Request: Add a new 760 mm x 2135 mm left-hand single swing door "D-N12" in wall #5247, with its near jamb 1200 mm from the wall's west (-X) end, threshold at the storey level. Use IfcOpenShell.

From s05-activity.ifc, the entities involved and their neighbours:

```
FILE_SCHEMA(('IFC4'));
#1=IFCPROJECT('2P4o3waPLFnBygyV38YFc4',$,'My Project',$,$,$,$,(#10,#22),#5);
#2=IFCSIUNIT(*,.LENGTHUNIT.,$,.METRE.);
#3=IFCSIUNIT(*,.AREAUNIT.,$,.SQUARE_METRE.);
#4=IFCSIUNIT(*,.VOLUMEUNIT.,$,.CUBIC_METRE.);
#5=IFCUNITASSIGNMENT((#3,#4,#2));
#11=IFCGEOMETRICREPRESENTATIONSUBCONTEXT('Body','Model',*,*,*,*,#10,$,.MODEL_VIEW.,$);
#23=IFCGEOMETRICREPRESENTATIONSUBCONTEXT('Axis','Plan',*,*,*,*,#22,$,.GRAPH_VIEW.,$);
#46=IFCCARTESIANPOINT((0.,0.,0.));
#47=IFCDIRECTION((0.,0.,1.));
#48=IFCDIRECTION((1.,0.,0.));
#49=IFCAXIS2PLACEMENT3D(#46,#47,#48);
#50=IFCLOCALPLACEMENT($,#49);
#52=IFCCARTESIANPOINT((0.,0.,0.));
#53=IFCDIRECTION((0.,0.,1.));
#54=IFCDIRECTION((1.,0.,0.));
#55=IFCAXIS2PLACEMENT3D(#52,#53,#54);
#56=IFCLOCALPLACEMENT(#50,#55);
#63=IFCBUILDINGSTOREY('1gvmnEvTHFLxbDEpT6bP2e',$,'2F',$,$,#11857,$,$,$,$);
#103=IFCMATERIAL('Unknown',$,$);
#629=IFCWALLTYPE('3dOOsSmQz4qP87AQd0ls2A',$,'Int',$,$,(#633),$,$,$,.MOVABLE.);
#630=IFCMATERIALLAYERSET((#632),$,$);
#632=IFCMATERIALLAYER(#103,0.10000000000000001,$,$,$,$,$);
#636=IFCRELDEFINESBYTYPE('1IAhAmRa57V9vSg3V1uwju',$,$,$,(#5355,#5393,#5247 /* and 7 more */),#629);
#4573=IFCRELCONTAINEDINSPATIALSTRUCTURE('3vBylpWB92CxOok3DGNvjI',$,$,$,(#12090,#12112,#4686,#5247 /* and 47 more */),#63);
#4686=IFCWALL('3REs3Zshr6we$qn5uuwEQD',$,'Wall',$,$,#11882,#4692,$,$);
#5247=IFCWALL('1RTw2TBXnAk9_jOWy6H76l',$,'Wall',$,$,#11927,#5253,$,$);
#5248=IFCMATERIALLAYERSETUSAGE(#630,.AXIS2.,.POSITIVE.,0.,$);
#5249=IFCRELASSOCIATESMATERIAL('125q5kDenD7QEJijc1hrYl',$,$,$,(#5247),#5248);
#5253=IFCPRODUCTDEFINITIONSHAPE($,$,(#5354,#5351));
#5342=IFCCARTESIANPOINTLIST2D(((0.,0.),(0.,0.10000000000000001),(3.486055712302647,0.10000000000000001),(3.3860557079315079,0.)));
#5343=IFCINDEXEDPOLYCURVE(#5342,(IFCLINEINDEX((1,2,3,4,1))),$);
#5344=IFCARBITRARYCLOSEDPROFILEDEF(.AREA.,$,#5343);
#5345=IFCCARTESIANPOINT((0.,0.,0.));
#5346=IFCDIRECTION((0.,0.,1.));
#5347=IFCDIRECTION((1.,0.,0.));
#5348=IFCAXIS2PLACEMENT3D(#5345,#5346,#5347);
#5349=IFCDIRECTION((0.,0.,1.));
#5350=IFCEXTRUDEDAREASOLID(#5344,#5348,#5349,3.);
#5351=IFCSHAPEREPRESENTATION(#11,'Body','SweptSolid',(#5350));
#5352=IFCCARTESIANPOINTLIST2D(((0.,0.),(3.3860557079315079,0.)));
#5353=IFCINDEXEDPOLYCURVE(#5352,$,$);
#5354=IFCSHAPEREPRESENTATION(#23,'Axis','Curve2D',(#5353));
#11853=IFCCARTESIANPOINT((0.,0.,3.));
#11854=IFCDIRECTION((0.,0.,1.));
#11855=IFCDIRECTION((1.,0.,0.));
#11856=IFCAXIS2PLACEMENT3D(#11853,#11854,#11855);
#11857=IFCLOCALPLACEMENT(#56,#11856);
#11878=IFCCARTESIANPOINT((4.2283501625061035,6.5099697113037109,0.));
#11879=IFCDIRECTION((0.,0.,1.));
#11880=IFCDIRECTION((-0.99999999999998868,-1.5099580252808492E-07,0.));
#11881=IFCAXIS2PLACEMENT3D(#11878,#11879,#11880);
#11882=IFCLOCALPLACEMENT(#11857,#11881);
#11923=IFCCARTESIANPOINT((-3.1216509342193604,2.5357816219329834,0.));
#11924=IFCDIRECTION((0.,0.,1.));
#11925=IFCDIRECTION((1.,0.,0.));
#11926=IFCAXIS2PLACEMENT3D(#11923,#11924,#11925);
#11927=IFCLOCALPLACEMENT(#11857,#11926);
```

```python
import numpy as np
import ifcopenshell
import ifcopenshell.api.feature
import ifcopenshell.api.geometry
import ifcopenshell.api.root
import ifcopenshell.api.spatial
import ifcopenshell.geom
import ifcopenshell.util.element
import ifcopenshell.util.placement
import ifcopenshell.util.representation
import ifcopenshell.util.shape
import ifcopenshell.util.unit

model = ifcopenshell.open("s05-activity.ifc")
unit_scale = ifcopenshell.util.unit.calculate_unit_scale(model)
settings = ifcopenshell.geom.settings()


def volume(element):
    """Net volume in cubic metres, openings subtracted."""
    shape = ifcopenshell.geom.create_shape(settings, element)
    return ifcopenshell.util.shape.get_volume(shape.geometry)


wall = model.by_guid("1RTw2TBXnAk9_jOWy6H76l")
storey = ifcopenshell.util.element.get_container(wall, ifc_class="IfcBuildingStorey")
context = ifcopenshell.util.representation.get_context(model, "Model", "Body", "MODEL_VIEW")
before = volume(wall)

width, height, from_end, sill = 0.76, 2.135, 1.2, 0.0  # metres

# The wall runs along its own X axis, and the end named is its -X end.
wall_shape = ifcopenshell.geom.create_shape(settings, wall)
x, y, z = ifcopenshell.util.shape.get_vertices(wall_shape.geometry).T
start = x.min() + from_end
face, thickness = float(y.min()), float(y.max() - y.min())
wall_matrix = ifcopenshell.util.placement.get_local_placement(wall.ObjectPlacement)
level = ifcopenshell.util.placement.get_local_placement(storey.ObjectPlacement)[2, 3]


def in_wall(x, y):
    """Placement at x, y metres in the wall's axes, at sill height."""
    matrix = wall_matrix.copy()
    matrix[:, 3] = wall_matrix @ np.array([x / unit_scale, y / unit_scale, 0.0, 1.0])
    matrix[2, 3] = level + sill / unit_scale
    return matrix


# Opening: a box that overshoots both wall faces by 50 mm.
opening = ifcopenshell.api.root.create_entity(model, ifc_class="IfcOpeningElement", predefined_type="OPENING")
box = ifcopenshell.api.geometry.add_wall_representation(
    model, context=context, length=width, height=height, thickness=thickness + 0.1
)
ifcopenshell.api.geometry.assign_representation(model, product=opening, representation=box)
ifcopenshell.api.geometry.edit_object_placement(model, product=opening, matrix=in_wall(start, face - 0.05), is_si=False)
ifcopenshell.api.feature.add_feature(model, feature=opening, element=wall)

door = ifcopenshell.api.root.create_entity(model, ifc_class="IfcDoor", name="D-N12", predefined_type="DOOR")
door.OverallWidth, door.OverallHeight = width / unit_scale, height / unit_scale
door.OperationType = "SINGLE_SWING_LEFT"
body = ifcopenshell.api.geometry.add_door_representation(
    model,
    context=context,
    overall_width=door.OverallWidth,
    overall_height=door.OverallHeight,
    operation_type="SINGLE_SWING_LEFT",
    lining_properties={"LiningDepth": thickness / unit_scale, "ThresholdDepth": thickness / unit_scale},
)
ifcopenshell.api.geometry.assign_representation(model, product=door, representation=body)
ifcopenshell.api.spatial.assign_container(model, products=[door], relating_structure=storey)
ifcopenshell.api.feature.add_filling(model, opening=opening, element=door)

# The lining spans the wall, so the door starts at the wall face.
ifcopenshell.api.geometry.edit_object_placement(model, product=door, matrix=in_wall(start, face), is_si=False)

after = volume(wall)

print(f"wall volume {before:.3f} -> {after:.3f} m3")

model.write("s05-activity-out.ifc")
```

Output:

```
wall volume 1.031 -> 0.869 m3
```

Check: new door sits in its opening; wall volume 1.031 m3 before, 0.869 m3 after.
